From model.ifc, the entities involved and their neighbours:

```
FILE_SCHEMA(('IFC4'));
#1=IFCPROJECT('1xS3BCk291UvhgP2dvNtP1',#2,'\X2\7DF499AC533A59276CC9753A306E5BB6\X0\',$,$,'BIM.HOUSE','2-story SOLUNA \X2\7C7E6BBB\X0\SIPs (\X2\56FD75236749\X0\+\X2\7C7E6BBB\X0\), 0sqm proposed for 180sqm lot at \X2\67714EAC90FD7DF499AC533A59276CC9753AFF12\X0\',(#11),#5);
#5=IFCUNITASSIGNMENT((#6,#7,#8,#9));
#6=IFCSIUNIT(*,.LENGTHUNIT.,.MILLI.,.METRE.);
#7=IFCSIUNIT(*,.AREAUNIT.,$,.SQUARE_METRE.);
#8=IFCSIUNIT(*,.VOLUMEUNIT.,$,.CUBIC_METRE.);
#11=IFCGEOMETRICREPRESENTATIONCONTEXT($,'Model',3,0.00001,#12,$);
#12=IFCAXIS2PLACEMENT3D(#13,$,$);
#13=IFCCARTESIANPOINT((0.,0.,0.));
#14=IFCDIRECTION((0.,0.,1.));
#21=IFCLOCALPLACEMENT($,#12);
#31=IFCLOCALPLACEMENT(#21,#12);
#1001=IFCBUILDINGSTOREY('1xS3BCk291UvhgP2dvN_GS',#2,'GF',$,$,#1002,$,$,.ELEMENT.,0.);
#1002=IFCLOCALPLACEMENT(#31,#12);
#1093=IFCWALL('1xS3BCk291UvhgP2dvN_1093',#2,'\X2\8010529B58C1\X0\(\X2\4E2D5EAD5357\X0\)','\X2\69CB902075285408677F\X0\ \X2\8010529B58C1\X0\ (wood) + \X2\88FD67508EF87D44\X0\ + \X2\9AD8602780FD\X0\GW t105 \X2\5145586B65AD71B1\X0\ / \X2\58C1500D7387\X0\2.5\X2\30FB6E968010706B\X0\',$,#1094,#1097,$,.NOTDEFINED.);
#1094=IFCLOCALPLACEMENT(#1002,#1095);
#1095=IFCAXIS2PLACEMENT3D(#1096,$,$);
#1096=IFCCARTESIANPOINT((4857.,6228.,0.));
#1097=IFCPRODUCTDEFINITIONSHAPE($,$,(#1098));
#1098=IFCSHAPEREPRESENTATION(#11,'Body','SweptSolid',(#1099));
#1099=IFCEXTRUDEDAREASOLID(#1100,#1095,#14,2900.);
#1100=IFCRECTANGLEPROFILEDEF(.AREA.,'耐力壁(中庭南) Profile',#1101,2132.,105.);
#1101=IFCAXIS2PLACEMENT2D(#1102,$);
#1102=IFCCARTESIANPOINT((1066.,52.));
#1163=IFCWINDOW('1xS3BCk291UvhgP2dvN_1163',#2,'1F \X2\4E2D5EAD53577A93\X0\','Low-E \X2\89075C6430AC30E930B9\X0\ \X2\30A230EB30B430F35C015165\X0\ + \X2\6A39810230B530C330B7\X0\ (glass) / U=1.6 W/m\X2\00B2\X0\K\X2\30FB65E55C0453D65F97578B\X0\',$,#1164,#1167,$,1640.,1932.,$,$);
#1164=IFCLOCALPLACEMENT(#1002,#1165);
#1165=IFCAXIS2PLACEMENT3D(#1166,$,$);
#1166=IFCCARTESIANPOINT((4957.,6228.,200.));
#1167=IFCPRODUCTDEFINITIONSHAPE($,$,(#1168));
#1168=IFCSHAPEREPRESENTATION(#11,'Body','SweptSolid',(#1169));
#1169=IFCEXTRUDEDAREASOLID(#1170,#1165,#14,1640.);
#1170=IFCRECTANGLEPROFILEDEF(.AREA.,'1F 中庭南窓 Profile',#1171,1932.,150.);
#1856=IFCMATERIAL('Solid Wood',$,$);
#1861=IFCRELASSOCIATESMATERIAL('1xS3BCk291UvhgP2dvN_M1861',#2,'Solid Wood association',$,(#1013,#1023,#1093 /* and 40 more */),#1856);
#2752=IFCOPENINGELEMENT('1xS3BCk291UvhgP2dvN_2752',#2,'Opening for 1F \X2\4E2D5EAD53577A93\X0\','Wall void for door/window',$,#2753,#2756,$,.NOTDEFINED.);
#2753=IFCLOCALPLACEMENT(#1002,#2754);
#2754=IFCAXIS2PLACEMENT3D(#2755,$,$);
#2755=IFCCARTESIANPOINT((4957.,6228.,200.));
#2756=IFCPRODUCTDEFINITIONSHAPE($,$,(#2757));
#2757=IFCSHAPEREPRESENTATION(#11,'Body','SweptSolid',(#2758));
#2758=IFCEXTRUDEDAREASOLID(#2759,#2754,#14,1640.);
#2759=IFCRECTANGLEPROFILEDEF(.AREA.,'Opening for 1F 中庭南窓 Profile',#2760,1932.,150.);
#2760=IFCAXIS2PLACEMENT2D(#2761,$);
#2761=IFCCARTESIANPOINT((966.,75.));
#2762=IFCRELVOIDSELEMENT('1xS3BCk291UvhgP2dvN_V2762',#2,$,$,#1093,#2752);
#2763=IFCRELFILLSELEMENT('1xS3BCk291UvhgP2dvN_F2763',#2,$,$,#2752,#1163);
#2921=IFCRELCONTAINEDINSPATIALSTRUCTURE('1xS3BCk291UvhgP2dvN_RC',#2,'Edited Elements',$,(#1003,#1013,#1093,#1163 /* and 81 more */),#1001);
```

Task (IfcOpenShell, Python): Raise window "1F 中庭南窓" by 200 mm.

```python
import numpy as np
import ifcopenshell
import ifcopenshell.api.geometry
import ifcopenshell.util.placement
import ifcopenshell.util.unit

model = ifcopenshell.open("model.ifc")
unit_scale = ifcopenshell.util.unit.calculate_unit_scale(model)

window = model.by_guid("1xS3BCk291UvhgP2dvN_1163")
opening = window.FillsVoids[0].RelatingOpeningElement
dz = 200.0

shift = np.array([0.0, 0.0, dz])
# The window is not placed relative to its opening, so move both.
for product in (opening, window):
    matrix = ifcopenshell.util.placement.get_local_placement(product.ObjectPlacement)
    matrix[:3, 3] += shift
    ifcopenshell.api.geometry.edit_object_placement(model, product=product, matrix=matrix, is_si=False)

print(f"moved by {dz * unit_scale:+.3f} m")

model.write("model-out.ifc")
```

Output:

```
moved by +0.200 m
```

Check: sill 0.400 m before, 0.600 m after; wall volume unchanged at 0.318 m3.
